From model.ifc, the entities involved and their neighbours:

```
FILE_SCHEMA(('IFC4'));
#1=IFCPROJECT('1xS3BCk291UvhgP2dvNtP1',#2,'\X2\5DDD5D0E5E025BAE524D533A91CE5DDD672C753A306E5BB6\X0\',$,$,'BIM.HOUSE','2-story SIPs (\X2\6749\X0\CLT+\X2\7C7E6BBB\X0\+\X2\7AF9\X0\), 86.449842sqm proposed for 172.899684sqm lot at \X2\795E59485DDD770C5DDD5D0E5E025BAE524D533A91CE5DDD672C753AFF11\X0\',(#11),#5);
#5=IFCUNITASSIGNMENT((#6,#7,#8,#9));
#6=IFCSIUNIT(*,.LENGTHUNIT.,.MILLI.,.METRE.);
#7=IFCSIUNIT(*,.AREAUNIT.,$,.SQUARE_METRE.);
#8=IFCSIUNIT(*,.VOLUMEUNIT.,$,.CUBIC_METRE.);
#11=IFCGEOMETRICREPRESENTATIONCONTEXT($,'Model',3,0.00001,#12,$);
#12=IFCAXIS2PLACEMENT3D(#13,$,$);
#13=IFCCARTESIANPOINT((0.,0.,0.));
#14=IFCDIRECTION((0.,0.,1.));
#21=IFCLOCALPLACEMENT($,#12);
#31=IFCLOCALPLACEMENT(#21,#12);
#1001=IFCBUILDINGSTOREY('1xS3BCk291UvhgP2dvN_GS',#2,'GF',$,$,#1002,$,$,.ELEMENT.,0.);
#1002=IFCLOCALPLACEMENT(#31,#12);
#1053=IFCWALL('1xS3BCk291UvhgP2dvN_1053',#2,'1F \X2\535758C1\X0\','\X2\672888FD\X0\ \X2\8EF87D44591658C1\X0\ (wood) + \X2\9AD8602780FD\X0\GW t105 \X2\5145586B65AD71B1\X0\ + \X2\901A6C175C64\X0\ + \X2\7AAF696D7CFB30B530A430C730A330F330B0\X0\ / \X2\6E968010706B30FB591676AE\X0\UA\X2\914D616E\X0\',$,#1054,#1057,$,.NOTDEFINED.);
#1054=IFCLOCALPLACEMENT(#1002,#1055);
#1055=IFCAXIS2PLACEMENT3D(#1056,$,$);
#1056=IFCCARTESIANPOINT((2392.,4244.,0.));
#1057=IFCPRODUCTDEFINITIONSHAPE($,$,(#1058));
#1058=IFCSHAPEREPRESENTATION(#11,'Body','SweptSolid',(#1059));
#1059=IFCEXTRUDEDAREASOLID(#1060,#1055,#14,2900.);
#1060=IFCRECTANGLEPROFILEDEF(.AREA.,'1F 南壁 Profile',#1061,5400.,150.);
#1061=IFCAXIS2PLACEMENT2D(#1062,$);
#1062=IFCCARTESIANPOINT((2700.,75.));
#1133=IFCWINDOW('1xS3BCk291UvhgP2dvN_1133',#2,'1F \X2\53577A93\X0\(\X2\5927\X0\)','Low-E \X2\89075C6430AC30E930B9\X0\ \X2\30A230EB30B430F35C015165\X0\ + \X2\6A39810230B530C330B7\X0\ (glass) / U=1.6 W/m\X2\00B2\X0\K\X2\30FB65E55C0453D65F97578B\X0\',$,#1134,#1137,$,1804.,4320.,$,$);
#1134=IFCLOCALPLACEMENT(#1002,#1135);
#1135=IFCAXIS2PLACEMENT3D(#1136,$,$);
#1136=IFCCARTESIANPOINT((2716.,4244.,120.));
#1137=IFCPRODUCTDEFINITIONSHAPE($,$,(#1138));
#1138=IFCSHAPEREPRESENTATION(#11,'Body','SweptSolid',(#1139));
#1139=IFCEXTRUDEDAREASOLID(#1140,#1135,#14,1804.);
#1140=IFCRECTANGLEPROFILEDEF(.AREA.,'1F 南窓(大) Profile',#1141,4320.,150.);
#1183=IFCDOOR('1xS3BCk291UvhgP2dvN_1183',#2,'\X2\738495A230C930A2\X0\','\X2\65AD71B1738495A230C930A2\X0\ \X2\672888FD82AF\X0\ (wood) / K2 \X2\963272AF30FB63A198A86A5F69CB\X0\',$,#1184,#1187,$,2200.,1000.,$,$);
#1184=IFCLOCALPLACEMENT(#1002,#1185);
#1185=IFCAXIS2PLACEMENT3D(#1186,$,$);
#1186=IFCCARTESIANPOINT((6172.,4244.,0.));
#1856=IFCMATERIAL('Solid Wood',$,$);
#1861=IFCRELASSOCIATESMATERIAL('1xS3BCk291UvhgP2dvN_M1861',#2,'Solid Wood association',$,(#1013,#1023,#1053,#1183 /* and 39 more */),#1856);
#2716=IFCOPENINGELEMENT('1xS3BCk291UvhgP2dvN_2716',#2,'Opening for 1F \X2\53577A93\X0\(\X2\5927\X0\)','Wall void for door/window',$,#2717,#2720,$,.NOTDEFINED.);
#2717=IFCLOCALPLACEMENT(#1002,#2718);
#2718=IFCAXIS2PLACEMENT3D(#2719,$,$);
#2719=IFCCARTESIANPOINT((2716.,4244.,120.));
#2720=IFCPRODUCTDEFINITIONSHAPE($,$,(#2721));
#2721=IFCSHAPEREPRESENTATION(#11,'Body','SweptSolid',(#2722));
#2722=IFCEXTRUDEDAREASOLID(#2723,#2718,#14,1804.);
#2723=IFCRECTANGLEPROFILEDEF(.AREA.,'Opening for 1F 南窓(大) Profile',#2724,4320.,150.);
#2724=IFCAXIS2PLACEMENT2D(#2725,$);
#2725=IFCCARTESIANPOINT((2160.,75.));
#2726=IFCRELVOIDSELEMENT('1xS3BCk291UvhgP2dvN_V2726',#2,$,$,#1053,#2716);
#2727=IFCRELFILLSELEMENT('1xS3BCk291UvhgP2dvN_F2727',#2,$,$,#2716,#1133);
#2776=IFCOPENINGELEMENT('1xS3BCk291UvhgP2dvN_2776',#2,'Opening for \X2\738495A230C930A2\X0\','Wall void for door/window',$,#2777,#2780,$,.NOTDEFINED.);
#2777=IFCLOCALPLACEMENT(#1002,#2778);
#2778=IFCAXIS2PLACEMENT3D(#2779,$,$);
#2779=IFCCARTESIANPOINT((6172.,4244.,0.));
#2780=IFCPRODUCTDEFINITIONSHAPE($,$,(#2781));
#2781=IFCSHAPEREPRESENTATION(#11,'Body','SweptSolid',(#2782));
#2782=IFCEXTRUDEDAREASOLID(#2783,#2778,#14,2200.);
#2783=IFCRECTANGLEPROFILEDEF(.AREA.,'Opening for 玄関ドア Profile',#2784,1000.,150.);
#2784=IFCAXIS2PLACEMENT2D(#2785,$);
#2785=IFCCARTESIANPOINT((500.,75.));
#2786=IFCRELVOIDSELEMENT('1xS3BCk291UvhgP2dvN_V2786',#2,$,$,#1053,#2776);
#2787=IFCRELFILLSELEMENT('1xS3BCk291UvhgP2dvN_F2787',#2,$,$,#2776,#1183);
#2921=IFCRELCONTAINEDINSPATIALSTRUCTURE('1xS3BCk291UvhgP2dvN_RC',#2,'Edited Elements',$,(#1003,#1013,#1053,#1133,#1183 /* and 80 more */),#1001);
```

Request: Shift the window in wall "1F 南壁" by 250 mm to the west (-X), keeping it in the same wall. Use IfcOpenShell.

```python
import ifcopenshell
import ifcopenshell.api.geometry
import ifcopenshell.util.placement
import ifcopenshell.util.unit

model = ifcopenshell.open("model.ifc")
unit_scale = ifcopenshell.util.unit.calculate_unit_scale(model)

window = model.by_guid("1xS3BCk291UvhgP2dvN_1133")
opening = window.FillsVoids[0].RelatingOpeningElement
wall = opening.VoidsElements[0].RelatingBuildingElement

wall_matrix = ifcopenshell.util.placement.get_local_placement(wall.ObjectPlacement)
shift = wall_matrix[:3, 0] * -0.25 / unit_scale
before = ifcopenshell.util.placement.get_local_placement(window.ObjectPlacement)[:3, 3].copy()

# The window is not placed relative to its opening, so move both.
for product in (opening, window):
    matrix = ifcopenshell.util.placement.get_local_placement(product.ObjectPlacement)
    matrix[:3, 3] += shift
    ifcopenshell.api.geometry.edit_object_placement(model, product=product, matrix=matrix, is_si=False)

after = ifcopenshell.util.placement.get_local_placement(window.ObjectPlacement)[:3, 3]
print("window moved by", (after - before).round(3) + 0.0)

model.write("model_rev.ifc")
```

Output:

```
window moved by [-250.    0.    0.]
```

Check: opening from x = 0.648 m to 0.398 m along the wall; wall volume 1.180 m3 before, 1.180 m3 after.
